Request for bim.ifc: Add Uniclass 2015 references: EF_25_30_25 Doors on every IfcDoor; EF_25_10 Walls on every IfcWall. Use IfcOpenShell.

First a look at what the model holds.

```python
import ifcopenshell

model = ifcopenshell.open("bim.ifc")
print(model.schema)
print("classifications:", [c.Name for c in model.by_type("IfcClassification")])
for ifc_class in ("IfcDoor", "IfcRoof", "IfcStair", "IfcWall", "IfcWindow"):
    print(ifc_class, len(model.by_type(ifc_class)))
```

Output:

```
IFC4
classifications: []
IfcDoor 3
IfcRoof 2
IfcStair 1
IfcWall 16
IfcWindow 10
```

```python
import ifcopenshell
import ifcopenshell.api.classification

model = ifcopenshell.open("bim.ifc")

system = ifcopenshell.api.classification.add_classification(model, classification="Uniclass 2015")

codes = {
    "IfcDoor": ("EF_25_30_25", "Doors"),
    "IfcWall": ("EF_25_10", "Walls"),
}
for ifc_class, (code, name) in codes.items():
    products = model.by_type(ifc_class)
    ifcopenshell.api.classification.add_reference(
        model, products=products, classification=system, identification=code, name=name
    )
    print(code, len(products))

model.write("bim_edited.ifc")
```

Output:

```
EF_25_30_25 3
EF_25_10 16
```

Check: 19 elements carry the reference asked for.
